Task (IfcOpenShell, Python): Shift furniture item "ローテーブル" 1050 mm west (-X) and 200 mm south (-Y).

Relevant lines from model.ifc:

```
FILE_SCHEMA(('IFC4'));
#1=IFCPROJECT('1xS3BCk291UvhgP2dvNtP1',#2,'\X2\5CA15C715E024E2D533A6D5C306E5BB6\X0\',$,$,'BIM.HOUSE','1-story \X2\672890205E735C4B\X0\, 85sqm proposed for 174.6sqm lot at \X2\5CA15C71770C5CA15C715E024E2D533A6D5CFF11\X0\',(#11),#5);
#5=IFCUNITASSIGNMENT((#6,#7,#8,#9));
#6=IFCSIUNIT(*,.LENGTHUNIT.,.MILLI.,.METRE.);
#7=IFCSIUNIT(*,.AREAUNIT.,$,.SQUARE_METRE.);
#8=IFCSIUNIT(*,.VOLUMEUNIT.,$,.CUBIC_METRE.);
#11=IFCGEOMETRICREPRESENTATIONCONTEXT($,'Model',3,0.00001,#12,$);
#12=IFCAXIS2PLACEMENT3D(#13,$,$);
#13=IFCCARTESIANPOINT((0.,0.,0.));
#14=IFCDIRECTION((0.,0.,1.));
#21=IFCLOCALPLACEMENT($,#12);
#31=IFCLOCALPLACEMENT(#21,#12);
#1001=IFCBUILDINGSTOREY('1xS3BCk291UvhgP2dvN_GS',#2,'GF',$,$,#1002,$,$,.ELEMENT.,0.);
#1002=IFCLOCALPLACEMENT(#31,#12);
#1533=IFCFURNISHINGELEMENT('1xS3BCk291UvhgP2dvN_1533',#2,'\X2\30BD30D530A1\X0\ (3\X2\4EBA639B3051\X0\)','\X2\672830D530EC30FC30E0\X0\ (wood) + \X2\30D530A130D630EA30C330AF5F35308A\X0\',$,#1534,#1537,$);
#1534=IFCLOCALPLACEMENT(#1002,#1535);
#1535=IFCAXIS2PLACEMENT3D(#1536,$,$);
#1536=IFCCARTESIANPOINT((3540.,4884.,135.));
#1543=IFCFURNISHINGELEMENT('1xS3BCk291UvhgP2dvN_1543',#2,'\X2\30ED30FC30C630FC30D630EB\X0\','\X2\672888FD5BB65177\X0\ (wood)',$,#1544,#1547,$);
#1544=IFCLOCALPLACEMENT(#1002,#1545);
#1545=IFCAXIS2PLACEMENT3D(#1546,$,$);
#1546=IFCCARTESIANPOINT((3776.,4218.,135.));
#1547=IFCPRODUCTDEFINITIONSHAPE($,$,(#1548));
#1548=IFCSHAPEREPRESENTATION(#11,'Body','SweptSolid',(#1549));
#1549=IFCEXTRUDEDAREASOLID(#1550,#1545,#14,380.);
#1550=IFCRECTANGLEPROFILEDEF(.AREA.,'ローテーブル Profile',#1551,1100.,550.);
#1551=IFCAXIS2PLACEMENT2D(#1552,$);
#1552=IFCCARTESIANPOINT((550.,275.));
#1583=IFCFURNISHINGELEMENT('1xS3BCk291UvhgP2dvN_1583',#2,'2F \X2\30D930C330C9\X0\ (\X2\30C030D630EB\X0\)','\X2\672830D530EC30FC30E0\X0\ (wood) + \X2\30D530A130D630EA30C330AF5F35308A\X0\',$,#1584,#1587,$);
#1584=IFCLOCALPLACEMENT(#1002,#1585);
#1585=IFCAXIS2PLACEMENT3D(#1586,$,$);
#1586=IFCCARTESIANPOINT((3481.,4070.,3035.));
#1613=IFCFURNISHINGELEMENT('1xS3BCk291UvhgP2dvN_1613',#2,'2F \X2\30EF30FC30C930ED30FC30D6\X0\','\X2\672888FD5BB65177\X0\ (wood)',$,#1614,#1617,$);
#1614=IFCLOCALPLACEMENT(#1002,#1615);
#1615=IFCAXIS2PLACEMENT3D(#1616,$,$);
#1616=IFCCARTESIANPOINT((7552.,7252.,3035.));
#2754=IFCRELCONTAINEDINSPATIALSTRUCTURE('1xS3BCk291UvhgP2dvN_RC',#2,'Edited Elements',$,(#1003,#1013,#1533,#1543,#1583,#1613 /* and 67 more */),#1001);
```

```python
import ifcopenshell
import ifcopenshell.api.geometry
import ifcopenshell.util.placement

model = ifcopenshell.open("model.ifc")

item = model.by_guid("1xS3BCk291UvhgP2dvN_1543")
matrix = ifcopenshell.util.placement.get_local_placement(item.ObjectPlacement)
matrix[0, 3] -= 1050.0
matrix[1, 3] -= 200.0
ifcopenshell.api.geometry.edit_object_placement(model, product=item, matrix=matrix, is_si=False)

print(ifcopenshell.util.placement.get_local_placement(item.ObjectPlacement).round(3) + 0.0)

model.write("model_updated.ifc")
```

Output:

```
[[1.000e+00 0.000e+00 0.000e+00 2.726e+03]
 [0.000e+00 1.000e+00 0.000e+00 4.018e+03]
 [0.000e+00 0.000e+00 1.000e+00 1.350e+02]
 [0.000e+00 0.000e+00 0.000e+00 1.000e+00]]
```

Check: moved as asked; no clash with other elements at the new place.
